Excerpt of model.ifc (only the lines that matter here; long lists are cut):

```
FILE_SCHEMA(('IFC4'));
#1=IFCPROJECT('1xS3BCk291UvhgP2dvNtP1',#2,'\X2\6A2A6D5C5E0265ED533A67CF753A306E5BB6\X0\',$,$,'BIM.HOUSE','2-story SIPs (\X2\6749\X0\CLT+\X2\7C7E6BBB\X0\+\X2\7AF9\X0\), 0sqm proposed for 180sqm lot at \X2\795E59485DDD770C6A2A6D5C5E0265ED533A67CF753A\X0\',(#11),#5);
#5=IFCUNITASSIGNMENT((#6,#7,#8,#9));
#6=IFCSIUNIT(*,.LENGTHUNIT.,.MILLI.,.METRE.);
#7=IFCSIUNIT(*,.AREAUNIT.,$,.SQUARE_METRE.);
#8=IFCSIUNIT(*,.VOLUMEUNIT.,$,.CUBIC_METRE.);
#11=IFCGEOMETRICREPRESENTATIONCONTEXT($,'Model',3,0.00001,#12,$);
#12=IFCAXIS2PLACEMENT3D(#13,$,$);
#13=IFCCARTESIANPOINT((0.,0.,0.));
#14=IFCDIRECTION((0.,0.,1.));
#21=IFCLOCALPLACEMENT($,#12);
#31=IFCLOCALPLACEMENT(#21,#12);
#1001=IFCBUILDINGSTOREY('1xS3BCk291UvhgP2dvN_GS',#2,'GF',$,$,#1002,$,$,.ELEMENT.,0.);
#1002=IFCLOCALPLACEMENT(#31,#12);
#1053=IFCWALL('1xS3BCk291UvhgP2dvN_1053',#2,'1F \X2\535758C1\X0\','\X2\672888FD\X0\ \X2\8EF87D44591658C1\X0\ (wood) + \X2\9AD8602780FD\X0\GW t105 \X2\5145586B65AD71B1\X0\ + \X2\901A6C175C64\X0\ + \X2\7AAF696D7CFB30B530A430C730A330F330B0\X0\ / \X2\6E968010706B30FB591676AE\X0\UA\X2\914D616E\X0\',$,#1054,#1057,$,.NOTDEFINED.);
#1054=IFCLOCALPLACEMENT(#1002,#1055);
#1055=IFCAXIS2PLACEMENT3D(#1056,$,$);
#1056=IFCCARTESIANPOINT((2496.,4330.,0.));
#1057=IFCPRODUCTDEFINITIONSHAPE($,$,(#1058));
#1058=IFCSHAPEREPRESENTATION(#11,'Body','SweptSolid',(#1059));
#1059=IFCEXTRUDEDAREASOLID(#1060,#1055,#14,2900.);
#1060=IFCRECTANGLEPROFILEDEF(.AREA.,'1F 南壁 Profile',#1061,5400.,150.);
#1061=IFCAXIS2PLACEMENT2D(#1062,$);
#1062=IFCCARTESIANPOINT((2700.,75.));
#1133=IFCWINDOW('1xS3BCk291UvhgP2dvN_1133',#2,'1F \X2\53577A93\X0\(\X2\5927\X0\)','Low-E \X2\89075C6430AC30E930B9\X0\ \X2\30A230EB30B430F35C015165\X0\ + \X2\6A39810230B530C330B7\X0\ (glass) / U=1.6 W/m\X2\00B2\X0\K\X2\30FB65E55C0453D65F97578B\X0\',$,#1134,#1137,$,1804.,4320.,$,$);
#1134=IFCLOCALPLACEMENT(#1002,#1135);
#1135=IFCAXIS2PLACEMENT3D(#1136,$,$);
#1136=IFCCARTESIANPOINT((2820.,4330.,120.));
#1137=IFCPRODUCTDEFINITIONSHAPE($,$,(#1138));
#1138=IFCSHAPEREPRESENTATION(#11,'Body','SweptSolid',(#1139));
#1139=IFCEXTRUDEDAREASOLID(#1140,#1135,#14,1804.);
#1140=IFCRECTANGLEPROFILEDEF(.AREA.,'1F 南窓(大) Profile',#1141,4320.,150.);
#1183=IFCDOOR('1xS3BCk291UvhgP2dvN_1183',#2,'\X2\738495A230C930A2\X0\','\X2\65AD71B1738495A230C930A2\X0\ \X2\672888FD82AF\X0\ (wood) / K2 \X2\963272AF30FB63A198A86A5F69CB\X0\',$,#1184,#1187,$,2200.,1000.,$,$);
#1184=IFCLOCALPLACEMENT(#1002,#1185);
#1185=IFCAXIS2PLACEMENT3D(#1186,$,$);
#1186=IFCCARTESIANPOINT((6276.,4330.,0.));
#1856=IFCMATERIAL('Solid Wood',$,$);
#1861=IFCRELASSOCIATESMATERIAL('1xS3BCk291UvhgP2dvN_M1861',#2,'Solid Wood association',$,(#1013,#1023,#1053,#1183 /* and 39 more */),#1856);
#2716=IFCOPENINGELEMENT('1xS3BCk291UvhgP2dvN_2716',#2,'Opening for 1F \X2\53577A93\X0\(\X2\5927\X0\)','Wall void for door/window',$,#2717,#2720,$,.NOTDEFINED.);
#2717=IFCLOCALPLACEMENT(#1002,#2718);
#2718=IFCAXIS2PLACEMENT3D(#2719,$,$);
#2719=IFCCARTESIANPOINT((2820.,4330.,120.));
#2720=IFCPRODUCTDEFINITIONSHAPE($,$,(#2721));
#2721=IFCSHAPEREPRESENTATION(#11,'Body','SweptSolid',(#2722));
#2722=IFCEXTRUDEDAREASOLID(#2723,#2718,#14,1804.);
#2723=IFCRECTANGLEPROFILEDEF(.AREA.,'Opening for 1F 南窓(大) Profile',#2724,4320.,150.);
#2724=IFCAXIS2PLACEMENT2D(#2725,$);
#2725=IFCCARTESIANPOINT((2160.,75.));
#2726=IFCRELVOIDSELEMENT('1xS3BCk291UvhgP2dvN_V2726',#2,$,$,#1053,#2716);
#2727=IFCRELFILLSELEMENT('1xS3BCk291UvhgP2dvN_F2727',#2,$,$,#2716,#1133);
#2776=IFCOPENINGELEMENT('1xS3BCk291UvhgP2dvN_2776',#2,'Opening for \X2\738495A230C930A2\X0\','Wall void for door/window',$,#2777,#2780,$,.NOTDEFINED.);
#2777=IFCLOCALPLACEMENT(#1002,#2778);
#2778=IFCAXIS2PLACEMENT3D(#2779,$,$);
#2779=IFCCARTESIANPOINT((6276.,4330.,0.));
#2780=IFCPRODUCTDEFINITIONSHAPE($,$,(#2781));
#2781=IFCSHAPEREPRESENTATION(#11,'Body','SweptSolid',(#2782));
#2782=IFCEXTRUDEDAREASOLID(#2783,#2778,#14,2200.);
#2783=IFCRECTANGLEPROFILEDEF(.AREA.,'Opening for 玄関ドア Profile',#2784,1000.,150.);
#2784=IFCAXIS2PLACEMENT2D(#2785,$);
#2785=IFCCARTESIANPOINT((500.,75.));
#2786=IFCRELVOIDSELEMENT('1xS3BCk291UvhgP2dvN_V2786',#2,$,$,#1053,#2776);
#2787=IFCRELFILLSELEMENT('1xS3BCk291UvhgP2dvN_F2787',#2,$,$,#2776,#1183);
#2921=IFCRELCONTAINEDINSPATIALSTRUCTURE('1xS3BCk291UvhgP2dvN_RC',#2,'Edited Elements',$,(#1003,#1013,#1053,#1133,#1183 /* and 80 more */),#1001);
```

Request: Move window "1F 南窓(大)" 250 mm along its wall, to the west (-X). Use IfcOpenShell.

```python
import ifcopenshell
import ifcopenshell.api.geometry
import ifcopenshell.util.placement
import ifcopenshell.util.unit

model = ifcopenshell.open("model.ifc")
unit_scale = ifcopenshell.util.unit.calculate_unit_scale(model)

window = model.by_guid("1xS3BCk291UvhgP2dvN_1133")
opening = window.FillsVoids[0].RelatingOpeningElement
wall = opening.VoidsElements[0].RelatingBuildingElement

wall_matrix = ifcopenshell.util.placement.get_local_placement(wall.ObjectPlacement)
shift = wall_matrix[:3, 0] * -0.25 / unit_scale
before = ifcopenshell.util.placement.get_local_placement(window.ObjectPlacement)[:3, 3].copy()

# The window is not placed relative to its opening, so move both.
for product in (opening, window):
    matrix = ifcopenshell.util.placement.get_local_placement(product.ObjectPlacement)
    matrix[:3, 3] += shift
    ifcopenshell.api.geometry.edit_object_placement(model, product=product, matrix=matrix, is_si=False)

after = ifcopenshell.util.placement.get_local_placement(window.ObjectPlacement)[:3, 3]
print("window moved by", (after - before).round(3) + 0.0)

model.write("model_edited.ifc")
```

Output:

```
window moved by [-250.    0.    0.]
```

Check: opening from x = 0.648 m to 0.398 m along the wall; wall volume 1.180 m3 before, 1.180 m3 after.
